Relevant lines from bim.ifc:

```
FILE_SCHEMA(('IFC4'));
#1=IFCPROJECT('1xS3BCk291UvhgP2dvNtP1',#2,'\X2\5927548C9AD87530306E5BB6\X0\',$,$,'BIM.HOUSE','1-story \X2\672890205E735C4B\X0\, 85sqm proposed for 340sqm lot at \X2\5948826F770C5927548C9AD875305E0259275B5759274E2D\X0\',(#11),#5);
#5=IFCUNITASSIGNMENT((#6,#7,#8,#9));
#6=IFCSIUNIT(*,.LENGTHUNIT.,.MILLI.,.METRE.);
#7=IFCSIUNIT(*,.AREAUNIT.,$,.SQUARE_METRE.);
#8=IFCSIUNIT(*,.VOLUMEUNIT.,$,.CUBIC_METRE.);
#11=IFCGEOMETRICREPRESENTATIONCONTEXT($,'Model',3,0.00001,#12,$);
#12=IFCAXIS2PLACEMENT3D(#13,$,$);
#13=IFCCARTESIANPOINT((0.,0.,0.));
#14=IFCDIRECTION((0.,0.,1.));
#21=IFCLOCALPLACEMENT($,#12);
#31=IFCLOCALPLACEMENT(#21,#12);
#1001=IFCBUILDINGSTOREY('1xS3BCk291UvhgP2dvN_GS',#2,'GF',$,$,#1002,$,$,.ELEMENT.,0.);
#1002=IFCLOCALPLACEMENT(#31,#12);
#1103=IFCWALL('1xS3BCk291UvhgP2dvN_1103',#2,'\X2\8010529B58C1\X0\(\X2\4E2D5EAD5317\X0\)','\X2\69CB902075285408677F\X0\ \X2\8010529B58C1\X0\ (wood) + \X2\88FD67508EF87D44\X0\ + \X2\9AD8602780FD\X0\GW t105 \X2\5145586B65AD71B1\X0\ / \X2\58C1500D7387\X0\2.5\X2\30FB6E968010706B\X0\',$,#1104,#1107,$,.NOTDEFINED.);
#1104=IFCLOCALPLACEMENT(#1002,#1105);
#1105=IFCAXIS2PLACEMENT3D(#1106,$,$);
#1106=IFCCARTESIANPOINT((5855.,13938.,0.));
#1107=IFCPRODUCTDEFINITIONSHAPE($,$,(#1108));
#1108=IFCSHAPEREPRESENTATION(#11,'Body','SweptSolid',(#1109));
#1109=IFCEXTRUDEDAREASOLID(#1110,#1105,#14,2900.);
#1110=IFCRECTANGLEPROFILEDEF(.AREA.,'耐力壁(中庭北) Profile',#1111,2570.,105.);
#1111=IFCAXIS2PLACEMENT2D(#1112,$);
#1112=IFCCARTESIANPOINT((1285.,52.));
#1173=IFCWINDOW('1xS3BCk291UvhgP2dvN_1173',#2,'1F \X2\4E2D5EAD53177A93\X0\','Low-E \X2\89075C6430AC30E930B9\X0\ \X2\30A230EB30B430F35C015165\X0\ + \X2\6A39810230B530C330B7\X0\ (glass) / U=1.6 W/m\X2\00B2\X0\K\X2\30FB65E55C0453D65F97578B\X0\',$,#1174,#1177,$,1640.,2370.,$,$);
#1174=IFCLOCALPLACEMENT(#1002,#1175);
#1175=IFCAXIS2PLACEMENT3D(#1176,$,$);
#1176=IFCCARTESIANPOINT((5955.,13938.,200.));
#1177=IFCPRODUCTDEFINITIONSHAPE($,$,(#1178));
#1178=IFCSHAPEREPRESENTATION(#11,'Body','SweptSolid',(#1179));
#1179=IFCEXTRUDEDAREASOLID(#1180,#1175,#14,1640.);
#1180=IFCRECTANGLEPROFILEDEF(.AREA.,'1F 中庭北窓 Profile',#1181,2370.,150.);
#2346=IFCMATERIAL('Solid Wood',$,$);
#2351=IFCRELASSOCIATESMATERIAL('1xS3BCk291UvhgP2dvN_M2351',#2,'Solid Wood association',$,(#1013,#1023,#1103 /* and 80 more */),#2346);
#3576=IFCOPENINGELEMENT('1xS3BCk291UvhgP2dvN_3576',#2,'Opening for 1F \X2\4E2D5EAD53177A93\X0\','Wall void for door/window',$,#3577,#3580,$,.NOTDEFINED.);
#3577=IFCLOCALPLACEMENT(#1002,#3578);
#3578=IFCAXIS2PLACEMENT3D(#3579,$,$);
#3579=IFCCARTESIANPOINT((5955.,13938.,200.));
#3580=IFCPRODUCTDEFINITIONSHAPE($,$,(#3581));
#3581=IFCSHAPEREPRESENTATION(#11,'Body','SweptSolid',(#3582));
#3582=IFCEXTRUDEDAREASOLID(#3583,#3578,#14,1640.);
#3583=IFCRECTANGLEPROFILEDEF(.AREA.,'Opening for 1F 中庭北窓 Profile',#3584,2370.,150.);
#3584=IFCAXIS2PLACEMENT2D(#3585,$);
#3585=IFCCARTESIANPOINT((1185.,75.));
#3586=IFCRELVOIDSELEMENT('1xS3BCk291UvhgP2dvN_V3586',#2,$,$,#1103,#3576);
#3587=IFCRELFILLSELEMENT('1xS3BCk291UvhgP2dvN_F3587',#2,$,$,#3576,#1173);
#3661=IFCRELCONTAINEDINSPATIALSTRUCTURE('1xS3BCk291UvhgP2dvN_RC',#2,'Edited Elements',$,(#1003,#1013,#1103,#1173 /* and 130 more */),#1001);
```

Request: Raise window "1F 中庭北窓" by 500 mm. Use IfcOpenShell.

```python
import numpy as np
import ifcopenshell
import ifcopenshell.api.geometry
import ifcopenshell.util.placement
import ifcopenshell.util.unit

model = ifcopenshell.open("bim.ifc")
unit_scale = ifcopenshell.util.unit.calculate_unit_scale(model)

window = model.by_guid("1xS3BCk291UvhgP2dvN_1173")
opening = window.FillsVoids[0].RelatingOpeningElement
dz = 0.5 / unit_scale

shift = np.array([0.0, 0.0, dz])
# The window is not placed relative to its opening, so move both.
for product in (opening, window):
    matrix = ifcopenshell.util.placement.get_local_placement(product.ObjectPlacement)
    matrix[:3, 3] += shift
    ifcopenshell.api.geometry.edit_object_placement(model, product=product, matrix=matrix, is_si=False)

print(f"moved by {dz * unit_scale:+.3f} m")

model.write("bim-out.ifc")
```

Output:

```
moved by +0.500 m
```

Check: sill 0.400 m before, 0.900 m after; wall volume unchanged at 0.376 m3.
